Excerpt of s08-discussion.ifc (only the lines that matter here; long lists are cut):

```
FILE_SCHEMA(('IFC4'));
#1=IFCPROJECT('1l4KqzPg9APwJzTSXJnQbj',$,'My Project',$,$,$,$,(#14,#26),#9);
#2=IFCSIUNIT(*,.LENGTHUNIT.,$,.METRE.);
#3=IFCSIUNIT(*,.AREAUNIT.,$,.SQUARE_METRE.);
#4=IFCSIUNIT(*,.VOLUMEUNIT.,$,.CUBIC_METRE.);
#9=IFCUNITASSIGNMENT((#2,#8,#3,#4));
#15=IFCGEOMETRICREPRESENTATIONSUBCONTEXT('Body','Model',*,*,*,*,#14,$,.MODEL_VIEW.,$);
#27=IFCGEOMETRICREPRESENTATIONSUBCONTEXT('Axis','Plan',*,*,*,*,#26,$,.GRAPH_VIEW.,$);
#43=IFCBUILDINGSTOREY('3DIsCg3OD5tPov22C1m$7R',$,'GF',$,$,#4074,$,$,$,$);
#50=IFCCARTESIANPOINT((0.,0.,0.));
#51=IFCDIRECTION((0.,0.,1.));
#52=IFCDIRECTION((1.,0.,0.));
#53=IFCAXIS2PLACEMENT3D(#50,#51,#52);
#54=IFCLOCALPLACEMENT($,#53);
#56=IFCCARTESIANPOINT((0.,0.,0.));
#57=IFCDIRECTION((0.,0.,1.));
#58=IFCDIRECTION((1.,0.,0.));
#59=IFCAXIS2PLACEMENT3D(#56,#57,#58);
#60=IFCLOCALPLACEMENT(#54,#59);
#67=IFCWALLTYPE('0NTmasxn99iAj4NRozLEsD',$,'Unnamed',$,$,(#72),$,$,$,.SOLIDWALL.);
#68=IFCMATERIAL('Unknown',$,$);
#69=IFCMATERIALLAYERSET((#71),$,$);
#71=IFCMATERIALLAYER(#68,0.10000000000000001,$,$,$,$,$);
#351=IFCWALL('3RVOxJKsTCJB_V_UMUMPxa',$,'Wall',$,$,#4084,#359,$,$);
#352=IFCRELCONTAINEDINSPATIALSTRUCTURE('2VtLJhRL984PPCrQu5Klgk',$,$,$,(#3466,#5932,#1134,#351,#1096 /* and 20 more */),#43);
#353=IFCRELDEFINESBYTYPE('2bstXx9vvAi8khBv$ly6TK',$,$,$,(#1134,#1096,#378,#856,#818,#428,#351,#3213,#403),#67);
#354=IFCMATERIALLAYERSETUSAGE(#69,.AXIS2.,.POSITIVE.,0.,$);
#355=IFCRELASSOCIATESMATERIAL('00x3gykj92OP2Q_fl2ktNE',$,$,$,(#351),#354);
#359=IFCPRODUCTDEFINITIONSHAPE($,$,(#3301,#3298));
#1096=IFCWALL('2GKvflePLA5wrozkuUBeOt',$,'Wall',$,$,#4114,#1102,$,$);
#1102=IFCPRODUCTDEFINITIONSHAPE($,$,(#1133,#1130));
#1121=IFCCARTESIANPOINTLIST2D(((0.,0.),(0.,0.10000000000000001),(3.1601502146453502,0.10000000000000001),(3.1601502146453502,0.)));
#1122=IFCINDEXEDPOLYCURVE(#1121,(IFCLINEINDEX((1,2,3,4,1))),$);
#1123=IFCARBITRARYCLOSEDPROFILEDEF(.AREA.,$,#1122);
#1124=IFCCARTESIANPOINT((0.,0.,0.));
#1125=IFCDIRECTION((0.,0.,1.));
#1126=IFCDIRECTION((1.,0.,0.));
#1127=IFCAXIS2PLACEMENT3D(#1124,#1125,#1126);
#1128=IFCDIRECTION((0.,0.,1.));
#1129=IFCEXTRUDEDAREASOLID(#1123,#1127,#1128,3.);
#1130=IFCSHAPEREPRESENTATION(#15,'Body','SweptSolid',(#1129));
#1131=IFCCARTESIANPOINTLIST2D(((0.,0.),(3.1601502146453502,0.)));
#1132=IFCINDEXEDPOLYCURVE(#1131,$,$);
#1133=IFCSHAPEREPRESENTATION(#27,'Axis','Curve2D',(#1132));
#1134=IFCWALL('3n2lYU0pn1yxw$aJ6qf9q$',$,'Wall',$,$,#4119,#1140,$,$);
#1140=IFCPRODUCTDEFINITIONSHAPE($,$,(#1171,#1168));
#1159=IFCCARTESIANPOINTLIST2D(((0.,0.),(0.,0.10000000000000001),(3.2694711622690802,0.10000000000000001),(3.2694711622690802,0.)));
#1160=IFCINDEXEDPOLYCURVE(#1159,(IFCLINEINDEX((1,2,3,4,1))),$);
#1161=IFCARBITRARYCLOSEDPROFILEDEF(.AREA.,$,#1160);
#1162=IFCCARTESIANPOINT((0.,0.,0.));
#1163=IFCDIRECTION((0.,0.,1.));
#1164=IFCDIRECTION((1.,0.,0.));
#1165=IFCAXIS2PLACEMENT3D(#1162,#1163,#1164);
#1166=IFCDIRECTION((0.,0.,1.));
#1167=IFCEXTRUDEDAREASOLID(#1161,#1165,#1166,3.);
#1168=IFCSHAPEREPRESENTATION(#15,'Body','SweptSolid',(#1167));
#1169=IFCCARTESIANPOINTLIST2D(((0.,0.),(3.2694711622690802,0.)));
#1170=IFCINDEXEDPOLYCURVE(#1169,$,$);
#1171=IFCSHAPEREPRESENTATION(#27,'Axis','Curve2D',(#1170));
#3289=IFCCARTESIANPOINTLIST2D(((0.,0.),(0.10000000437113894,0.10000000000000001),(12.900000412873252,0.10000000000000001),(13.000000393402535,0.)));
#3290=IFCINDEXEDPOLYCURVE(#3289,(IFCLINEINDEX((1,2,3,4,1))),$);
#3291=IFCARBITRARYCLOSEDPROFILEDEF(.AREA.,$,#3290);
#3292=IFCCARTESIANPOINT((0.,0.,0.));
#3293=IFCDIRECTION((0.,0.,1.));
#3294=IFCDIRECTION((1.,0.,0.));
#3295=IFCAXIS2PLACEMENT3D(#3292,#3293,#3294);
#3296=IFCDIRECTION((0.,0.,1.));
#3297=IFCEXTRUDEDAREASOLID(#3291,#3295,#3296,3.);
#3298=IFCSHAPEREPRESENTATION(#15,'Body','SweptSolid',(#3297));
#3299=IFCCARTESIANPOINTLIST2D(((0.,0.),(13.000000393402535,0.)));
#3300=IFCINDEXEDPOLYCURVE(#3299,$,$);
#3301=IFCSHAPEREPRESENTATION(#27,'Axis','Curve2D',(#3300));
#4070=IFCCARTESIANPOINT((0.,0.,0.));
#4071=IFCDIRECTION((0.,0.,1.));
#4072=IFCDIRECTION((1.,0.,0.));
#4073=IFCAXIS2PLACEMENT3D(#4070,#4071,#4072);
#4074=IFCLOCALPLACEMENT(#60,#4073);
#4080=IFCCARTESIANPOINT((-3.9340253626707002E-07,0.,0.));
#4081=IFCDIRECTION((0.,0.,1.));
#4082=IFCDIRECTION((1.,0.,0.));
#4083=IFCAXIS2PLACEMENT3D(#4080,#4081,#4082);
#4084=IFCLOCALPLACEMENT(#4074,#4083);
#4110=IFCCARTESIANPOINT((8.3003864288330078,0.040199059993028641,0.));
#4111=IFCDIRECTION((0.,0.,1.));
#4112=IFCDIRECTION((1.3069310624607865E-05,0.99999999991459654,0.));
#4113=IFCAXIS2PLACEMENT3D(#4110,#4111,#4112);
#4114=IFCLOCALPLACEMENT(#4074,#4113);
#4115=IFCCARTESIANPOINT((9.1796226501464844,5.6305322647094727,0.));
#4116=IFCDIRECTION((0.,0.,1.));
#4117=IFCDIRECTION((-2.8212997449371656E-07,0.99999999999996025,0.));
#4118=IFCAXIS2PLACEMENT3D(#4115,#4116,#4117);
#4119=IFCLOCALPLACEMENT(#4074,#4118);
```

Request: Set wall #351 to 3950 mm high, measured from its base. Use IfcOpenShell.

```python
import ifcopenshell
import ifcopenshell.geom
import ifcopenshell.util.representation
import ifcopenshell.util.shape
import ifcopenshell.util.unit

model = ifcopenshell.open("s08-discussion.ifc")
unit_scale = ifcopenshell.util.unit.calculate_unit_scale(model)
settings = ifcopenshell.geom.settings()


def volume(element):
    """Net volume in cubic metres, openings subtracted."""
    shape = ifcopenshell.geom.create_shape(settings, element)
    return ifcopenshell.util.shape.get_volume(shape.geometry)


wall = model.by_guid("3RVOxJKsTCJB_V_UMUMPxa")
before = volume(wall)

body = ifcopenshell.util.representation.get_representation(wall, "Model", "Body")
solid = body.Items[0]
old_height = solid.Depth
solid.Depth = 3.95 / unit_scale
after = volume(wall)

print(f"height {old_height:g} -> {solid.Depth:g}, volume {before:.3f} -> {after:.3f} m3")

model.write("s08-discussion_rev.ifc")
```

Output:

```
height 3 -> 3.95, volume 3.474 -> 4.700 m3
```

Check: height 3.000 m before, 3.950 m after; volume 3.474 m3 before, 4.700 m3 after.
